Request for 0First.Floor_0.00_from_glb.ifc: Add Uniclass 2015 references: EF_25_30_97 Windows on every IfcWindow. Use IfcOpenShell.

First a look at what the model holds.

```python
import ifcopenshell

model = ifcopenshell.open("0First.Floor_0.00_from_glb.ifc")
print(model.schema)
print("classifications:", [c.Name for c in model.by_type("IfcClassification")])
for ifc_class in ("IfcDoor", "IfcRoof", "IfcStair", "IfcWall", "IfcWindow"):
    print(ifc_class, len(model.by_type(ifc_class)))
```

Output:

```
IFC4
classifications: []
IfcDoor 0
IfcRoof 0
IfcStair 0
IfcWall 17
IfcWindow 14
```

```python
import ifcopenshell
import ifcopenshell.api.classification

model = ifcopenshell.open("0First.Floor_0.00_from_glb.ifc")

system = ifcopenshell.api.classification.add_classification(model, classification="Uniclass 2015")

codes = {
    "IfcWindow": ("EF_25_30_97", "Windows"),
}
for ifc_class, (code, name) in codes.items():
    products = model.by_type(ifc_class)
    ifcopenshell.api.classification.add_reference(
        model, products=products, classification=system, identification=code, name=name
    )
    print(code, len(products))

model.write("0First.Floor_0.00_from_glb_edited.ifc")
```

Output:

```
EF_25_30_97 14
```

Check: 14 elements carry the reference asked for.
